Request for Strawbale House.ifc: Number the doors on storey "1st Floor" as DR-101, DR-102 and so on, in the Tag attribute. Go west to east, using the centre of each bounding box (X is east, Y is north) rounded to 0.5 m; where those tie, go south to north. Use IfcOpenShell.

First a look at what the model holds.

```python
import ifcopenshell
import ifcopenshell.util.element
import ifcopenshell.util.placement

model = ifcopenshell.open("Strawbale House.ifc")
print(model.schema)
storey = next(s for s in model.by_type("IfcBuildingStorey") if s.Name == "1st Floor")
doors = [e for e in ifcopenshell.util.element.get_decomposition(storey) if e.is_a("IfcDoor")]
for e in sorted(doors, key=lambda e: e.id()):
    origin = ifcopenshell.util.placement.get_local_placement(e.ObjectPlacement)[:3, 3]
    print(e.id(), e.Tag, e.Name, origin.round(2) + 0.0, sep=" | ")
```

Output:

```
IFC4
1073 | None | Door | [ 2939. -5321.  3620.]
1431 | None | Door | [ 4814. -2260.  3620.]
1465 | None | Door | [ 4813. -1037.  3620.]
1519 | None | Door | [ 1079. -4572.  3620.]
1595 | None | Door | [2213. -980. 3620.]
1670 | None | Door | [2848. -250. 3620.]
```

```python
import ifcopenshell
import ifcopenshell.geom
import ifcopenshell.util.element
import ifcopenshell.util.shape

model = ifcopenshell.open("Strawbale House.ifc")
settings = ifcopenshell.geom.settings()
settings.set("use-world-coords", True)


def centre(element):
    shape = ifcopenshell.geom.create_shape(settings, element)
    return ifcopenshell.util.shape.get_bbox_centroid(shape.geometry)


storey = next(s for s in model.by_type("IfcBuildingStorey") if s.Name == "1st Floor")
doors = [e for e in ifcopenshell.util.element.get_decomposition(storey) if e.is_a("IfcDoor")]

# Insertion points can sit at a corner or the storey origin, so sort by the geometry (in metres).
centres = {e: centre(e) for e in doors}
doors.sort(key=lambda e: (round(centres[e][0] / 0.5), centres[e][1]))

for i, e in enumerate(doors, start=1):
    number = f"DR-1{i:02d}"
    e.Tag = number
    print(e.id(), number)

model.write("Strawbale House_updated.ifc")
```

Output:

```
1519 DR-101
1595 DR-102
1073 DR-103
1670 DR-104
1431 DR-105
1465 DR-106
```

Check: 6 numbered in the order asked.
